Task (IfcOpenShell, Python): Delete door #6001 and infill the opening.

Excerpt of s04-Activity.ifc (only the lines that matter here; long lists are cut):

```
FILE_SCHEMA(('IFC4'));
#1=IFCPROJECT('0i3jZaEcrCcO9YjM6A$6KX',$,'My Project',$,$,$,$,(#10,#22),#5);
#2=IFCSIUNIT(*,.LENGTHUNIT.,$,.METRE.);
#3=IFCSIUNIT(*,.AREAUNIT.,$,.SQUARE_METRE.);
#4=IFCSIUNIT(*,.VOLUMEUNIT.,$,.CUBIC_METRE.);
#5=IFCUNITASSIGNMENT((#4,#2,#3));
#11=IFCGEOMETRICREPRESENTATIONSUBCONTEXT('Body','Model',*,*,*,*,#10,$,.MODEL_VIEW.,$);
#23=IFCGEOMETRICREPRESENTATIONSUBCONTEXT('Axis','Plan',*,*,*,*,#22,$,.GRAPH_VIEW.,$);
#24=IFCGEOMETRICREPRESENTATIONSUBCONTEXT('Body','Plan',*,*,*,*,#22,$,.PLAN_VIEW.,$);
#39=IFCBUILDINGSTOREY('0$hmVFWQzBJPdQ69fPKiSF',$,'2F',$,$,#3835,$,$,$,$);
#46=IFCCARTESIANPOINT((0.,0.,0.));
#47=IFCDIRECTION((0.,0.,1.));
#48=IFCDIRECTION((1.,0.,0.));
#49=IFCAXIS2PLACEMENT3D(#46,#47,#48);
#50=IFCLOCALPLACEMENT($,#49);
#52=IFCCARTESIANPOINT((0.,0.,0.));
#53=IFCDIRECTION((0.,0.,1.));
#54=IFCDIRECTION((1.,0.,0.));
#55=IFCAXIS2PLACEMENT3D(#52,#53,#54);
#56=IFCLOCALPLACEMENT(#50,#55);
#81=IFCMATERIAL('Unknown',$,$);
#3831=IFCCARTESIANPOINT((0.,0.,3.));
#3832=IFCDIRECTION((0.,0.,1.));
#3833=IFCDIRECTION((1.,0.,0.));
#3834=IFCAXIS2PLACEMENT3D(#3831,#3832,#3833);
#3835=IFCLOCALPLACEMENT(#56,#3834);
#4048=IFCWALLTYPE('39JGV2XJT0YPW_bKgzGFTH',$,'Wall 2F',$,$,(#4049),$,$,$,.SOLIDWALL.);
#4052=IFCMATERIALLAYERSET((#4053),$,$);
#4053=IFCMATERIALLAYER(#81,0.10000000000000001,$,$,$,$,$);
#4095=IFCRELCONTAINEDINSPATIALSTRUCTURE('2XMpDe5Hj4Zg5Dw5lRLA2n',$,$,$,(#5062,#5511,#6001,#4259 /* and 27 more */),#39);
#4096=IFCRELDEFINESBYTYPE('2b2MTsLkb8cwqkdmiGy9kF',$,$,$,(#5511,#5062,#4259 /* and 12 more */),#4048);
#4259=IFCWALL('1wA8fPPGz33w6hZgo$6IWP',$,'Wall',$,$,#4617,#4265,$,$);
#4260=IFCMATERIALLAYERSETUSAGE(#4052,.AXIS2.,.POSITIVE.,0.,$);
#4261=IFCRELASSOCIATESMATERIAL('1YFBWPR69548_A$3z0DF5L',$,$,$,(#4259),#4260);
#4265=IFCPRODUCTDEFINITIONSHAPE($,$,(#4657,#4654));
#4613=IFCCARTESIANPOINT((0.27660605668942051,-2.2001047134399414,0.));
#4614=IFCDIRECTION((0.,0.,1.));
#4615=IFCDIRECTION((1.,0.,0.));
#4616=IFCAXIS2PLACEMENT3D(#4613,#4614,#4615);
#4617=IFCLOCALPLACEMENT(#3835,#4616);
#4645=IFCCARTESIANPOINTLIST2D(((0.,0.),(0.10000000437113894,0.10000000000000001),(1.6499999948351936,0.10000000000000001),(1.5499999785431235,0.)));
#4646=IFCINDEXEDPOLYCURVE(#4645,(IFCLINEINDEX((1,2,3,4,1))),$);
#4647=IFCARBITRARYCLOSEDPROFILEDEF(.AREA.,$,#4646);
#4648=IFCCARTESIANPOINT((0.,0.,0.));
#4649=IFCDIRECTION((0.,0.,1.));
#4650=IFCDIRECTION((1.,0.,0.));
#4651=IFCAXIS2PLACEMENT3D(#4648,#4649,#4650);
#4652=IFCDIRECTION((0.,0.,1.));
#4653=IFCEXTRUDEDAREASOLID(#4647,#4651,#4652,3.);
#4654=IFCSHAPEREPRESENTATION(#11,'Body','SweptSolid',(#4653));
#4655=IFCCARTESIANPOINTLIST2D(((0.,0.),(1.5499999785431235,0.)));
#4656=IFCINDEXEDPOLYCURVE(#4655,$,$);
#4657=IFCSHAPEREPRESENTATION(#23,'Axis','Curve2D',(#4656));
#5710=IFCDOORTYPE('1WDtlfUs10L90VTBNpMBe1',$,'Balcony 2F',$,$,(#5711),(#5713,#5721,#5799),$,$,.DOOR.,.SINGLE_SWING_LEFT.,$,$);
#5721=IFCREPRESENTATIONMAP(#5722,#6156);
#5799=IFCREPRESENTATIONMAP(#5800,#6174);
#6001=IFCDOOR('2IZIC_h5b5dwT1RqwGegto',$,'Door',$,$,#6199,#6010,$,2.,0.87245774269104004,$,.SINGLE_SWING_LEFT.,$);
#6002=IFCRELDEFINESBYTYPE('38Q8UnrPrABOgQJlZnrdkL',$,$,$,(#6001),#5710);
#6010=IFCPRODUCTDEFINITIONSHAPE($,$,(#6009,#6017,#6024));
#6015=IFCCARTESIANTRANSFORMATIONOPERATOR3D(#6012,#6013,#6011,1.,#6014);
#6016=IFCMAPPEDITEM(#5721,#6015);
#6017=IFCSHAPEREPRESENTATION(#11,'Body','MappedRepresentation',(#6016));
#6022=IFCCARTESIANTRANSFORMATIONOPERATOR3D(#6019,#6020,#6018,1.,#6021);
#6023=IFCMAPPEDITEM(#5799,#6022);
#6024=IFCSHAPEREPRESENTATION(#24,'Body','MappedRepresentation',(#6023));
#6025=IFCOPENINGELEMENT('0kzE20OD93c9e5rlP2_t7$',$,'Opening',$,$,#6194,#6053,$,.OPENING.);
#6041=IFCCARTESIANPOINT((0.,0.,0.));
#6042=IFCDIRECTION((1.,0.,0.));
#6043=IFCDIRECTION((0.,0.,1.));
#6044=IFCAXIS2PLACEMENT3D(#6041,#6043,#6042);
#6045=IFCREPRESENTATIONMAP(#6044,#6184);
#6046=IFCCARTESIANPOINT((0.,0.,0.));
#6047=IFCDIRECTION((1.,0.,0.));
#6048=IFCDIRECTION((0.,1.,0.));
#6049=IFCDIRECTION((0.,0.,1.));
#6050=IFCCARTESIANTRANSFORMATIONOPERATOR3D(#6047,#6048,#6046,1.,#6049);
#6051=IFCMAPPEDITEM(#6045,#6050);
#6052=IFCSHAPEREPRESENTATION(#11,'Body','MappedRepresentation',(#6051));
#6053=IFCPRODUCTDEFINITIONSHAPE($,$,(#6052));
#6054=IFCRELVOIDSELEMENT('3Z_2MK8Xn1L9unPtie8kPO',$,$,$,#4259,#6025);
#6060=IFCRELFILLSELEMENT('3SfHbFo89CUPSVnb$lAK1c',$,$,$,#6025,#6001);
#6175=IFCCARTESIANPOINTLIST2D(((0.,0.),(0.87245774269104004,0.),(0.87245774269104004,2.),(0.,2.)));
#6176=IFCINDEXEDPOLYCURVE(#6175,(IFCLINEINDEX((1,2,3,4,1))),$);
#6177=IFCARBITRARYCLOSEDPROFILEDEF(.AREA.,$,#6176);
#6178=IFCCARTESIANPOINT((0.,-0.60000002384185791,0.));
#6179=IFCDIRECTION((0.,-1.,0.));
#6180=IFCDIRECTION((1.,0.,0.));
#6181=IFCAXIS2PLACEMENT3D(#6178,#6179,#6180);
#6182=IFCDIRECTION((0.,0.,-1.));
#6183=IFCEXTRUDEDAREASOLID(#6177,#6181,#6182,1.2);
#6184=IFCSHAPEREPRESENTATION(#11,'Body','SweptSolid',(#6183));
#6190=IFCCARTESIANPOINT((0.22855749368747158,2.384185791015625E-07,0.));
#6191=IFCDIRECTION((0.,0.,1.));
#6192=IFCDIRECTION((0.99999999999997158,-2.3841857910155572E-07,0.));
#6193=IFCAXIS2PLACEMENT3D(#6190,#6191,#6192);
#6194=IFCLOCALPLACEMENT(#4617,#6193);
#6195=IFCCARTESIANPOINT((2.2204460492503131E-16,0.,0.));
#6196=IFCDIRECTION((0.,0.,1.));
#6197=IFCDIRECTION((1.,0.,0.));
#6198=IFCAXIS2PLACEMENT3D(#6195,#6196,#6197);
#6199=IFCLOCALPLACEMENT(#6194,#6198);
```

```python
import ifcopenshell
import ifcopenshell.api.feature
import ifcopenshell.api.root
import ifcopenshell.geom
import ifcopenshell.util.shape

model = ifcopenshell.open("s04-Activity.ifc")
settings = ifcopenshell.geom.settings()


def volume(element):
    """Net volume in cubic metres, openings subtracted."""
    shape = ifcopenshell.geom.create_shape(settings, element)
    return ifcopenshell.util.shape.get_volume(shape.geometry)


door = model.by_guid("2IZIC_h5b5dwT1RqwGegto")
opening = door.FillsVoids[0].RelatingOpeningElement
wall = opening.VoidsElements[0].RelatingBuildingElement
before = volume(wall)

ifcopenshell.api.root.remove_product(model, product=door)
ifcopenshell.api.feature.remove_feature(model, feature=opening)

after = volume(wall)

print(f"wall volume {before:.3f} -> {after:.3f} m3")

model.write("s04-Activity_rev.ifc")
```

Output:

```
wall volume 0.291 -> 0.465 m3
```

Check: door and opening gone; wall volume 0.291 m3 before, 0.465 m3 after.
